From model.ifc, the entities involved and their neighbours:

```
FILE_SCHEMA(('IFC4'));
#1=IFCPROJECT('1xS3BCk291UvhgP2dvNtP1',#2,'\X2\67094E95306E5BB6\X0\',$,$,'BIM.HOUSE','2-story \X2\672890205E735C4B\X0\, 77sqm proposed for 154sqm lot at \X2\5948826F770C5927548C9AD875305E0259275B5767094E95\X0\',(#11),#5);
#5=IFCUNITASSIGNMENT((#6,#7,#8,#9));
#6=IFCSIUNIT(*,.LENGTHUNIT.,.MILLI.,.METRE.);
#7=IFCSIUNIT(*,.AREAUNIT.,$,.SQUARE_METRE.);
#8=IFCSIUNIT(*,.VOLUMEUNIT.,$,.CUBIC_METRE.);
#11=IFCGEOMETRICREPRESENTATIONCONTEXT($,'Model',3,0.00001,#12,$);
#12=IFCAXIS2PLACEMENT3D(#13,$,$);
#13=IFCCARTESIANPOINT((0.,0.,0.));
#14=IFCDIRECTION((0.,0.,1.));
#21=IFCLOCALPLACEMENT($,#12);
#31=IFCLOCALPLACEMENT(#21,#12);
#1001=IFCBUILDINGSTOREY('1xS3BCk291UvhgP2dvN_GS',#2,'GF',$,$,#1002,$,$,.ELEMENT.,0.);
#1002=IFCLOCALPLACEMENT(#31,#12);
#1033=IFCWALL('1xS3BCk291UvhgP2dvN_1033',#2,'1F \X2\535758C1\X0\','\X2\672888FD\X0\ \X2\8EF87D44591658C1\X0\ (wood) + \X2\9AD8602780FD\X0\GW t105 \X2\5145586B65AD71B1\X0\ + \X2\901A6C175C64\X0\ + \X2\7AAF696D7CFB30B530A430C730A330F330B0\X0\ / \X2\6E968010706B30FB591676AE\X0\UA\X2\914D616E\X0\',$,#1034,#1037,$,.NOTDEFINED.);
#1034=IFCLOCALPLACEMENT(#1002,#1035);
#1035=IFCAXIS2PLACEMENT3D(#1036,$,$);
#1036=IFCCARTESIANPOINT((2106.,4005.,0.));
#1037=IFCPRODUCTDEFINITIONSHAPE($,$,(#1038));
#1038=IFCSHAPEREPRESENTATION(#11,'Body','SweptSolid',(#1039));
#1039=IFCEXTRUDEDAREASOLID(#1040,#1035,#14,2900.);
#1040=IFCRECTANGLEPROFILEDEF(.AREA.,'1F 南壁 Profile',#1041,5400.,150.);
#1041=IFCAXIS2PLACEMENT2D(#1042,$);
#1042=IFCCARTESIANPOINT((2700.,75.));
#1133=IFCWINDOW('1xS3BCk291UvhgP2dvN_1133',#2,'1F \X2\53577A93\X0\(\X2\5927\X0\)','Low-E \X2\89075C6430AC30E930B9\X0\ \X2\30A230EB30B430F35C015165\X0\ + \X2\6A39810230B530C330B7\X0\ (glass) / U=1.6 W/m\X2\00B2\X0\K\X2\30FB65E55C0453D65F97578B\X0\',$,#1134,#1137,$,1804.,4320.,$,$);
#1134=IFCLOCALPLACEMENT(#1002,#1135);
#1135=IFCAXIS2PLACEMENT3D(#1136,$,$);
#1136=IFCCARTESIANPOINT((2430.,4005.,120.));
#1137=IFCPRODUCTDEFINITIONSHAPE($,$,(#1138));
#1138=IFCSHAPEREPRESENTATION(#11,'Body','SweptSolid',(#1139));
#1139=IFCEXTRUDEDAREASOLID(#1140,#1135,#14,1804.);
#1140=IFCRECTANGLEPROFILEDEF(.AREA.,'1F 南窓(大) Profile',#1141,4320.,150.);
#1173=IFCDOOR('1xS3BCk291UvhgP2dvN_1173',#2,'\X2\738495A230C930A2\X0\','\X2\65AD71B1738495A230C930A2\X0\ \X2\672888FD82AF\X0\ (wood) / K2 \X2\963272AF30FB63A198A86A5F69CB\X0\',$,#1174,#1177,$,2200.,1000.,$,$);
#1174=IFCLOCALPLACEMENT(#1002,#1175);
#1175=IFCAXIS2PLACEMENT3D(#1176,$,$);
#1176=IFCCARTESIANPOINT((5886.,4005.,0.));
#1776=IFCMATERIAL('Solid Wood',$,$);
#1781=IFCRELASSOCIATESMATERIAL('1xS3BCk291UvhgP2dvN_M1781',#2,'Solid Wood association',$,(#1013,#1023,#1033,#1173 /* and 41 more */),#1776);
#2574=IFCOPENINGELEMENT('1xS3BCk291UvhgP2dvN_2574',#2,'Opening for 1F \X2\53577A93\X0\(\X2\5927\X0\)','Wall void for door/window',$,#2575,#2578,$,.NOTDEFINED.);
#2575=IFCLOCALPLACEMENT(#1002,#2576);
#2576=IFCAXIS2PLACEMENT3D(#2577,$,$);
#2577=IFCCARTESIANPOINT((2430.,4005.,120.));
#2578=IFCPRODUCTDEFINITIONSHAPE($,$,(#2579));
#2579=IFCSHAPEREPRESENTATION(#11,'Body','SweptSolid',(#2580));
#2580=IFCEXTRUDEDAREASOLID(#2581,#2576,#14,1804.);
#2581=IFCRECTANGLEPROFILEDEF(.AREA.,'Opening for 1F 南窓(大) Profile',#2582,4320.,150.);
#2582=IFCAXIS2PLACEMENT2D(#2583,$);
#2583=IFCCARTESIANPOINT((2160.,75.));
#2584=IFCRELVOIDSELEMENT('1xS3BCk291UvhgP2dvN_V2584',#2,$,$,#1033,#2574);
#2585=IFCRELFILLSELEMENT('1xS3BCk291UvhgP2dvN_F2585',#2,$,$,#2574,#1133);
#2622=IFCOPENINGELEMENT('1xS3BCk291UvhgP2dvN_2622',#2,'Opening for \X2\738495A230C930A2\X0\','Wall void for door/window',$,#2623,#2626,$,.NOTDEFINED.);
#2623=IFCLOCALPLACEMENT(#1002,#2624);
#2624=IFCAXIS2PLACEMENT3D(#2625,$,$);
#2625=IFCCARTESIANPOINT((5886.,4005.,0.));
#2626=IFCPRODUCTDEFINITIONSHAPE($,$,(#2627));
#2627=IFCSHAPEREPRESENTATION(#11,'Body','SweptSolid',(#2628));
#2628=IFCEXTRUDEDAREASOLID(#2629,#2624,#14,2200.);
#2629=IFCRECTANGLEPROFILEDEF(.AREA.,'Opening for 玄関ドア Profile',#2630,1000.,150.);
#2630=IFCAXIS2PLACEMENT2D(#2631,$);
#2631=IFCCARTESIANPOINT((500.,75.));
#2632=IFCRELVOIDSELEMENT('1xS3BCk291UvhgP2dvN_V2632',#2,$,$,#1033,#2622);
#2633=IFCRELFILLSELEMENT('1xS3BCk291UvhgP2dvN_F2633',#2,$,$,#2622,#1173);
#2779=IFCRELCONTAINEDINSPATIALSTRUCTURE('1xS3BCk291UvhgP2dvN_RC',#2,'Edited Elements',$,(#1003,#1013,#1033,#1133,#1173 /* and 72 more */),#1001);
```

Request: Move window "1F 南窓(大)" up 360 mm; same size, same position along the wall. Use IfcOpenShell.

```python
import numpy as np
import ifcopenshell
import ifcopenshell.api.geometry
import ifcopenshell.util.placement
import ifcopenshell.util.unit

model = ifcopenshell.open("model.ifc")
unit_scale = ifcopenshell.util.unit.calculate_unit_scale(model)

window = model.by_guid("1xS3BCk291UvhgP2dvN_1133")
opening = window.FillsVoids[0].RelatingOpeningElement
dz = 360.0

shift = np.array([0.0, 0.0, dz])
# The window is not placed relative to its opening, so move both.
for product in (opening, window):
    matrix = ifcopenshell.util.placement.get_local_placement(product.ObjectPlacement)
    matrix[:3, 3] += shift
    ifcopenshell.api.geometry.edit_object_placement(model, product=product, matrix=matrix, is_si=False)

print(f"moved by {dz * unit_scale:+.3f} m")

model.write("model_edited.ifc")
```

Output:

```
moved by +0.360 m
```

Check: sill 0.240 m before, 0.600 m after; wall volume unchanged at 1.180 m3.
